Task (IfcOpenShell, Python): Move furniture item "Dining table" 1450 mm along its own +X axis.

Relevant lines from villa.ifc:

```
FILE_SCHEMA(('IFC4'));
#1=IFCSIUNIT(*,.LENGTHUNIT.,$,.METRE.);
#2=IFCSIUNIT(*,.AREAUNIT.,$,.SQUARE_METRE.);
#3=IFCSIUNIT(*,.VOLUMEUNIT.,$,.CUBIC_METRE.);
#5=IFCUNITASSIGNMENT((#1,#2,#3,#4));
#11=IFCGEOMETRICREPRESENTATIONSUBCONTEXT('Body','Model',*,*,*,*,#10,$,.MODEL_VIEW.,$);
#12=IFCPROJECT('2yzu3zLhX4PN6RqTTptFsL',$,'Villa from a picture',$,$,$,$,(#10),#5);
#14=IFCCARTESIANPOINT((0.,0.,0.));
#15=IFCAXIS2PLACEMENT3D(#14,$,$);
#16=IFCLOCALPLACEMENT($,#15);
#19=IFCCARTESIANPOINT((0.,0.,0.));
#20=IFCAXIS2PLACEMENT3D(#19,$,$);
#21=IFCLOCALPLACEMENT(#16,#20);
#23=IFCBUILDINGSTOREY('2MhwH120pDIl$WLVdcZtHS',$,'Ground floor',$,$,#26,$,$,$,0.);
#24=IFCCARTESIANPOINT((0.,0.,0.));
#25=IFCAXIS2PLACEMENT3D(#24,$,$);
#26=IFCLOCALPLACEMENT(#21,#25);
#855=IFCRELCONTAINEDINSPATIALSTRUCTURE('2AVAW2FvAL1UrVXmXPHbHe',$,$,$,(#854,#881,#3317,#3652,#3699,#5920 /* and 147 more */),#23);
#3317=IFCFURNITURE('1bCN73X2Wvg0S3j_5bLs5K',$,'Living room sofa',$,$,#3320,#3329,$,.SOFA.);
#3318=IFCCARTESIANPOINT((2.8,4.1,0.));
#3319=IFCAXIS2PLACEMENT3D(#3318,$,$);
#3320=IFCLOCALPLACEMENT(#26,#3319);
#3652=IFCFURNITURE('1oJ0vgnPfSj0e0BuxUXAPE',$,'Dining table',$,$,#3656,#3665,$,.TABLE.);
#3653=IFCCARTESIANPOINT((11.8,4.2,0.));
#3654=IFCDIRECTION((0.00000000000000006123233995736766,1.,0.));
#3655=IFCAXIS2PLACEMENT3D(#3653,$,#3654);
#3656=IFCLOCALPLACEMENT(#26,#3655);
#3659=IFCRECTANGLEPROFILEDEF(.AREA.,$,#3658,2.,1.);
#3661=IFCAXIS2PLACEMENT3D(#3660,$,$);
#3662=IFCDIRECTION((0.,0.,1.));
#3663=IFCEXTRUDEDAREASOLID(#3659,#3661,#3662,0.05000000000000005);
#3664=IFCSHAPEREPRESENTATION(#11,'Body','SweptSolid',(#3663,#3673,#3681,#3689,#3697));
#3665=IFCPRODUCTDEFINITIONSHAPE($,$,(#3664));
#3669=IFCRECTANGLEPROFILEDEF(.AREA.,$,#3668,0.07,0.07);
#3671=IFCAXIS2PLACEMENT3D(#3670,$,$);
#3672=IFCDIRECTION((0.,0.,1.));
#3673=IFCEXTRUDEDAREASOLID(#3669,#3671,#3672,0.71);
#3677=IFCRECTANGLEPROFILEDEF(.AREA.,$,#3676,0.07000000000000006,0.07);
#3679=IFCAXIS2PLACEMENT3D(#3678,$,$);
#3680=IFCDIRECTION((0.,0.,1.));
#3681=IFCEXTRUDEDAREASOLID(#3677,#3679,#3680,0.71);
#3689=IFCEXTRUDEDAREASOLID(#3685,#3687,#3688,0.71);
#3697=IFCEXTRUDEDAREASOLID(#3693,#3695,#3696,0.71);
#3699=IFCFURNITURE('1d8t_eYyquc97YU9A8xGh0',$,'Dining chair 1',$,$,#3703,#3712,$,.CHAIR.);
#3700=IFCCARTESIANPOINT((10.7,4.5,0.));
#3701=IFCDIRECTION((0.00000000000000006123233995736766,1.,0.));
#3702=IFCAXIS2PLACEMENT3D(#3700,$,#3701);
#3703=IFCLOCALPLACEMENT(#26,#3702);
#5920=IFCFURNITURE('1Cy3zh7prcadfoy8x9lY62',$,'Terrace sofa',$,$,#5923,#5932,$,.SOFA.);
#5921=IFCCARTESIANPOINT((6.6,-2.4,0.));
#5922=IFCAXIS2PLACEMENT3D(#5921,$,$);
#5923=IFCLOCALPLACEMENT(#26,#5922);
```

```python
import ifcopenshell
import ifcopenshell.api.geometry
import ifcopenshell.util.placement

model = ifcopenshell.open("villa.ifc")

item = model.by_id(3652)
matrix = ifcopenshell.util.placement.get_local_placement(item.ObjectPlacement)
matrix[:3, 3] += matrix[:3, 0] * 1.45
ifcopenshell.api.geometry.edit_object_placement(model, product=item, matrix=matrix, is_si=False)

print(ifcopenshell.util.placement.get_local_placement(item.ObjectPlacement).round(3) + 0.0)

model.write("villa_v2.ifc")
```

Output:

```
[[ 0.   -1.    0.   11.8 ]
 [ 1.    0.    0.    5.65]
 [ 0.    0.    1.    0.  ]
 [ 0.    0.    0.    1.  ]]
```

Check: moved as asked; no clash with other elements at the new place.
